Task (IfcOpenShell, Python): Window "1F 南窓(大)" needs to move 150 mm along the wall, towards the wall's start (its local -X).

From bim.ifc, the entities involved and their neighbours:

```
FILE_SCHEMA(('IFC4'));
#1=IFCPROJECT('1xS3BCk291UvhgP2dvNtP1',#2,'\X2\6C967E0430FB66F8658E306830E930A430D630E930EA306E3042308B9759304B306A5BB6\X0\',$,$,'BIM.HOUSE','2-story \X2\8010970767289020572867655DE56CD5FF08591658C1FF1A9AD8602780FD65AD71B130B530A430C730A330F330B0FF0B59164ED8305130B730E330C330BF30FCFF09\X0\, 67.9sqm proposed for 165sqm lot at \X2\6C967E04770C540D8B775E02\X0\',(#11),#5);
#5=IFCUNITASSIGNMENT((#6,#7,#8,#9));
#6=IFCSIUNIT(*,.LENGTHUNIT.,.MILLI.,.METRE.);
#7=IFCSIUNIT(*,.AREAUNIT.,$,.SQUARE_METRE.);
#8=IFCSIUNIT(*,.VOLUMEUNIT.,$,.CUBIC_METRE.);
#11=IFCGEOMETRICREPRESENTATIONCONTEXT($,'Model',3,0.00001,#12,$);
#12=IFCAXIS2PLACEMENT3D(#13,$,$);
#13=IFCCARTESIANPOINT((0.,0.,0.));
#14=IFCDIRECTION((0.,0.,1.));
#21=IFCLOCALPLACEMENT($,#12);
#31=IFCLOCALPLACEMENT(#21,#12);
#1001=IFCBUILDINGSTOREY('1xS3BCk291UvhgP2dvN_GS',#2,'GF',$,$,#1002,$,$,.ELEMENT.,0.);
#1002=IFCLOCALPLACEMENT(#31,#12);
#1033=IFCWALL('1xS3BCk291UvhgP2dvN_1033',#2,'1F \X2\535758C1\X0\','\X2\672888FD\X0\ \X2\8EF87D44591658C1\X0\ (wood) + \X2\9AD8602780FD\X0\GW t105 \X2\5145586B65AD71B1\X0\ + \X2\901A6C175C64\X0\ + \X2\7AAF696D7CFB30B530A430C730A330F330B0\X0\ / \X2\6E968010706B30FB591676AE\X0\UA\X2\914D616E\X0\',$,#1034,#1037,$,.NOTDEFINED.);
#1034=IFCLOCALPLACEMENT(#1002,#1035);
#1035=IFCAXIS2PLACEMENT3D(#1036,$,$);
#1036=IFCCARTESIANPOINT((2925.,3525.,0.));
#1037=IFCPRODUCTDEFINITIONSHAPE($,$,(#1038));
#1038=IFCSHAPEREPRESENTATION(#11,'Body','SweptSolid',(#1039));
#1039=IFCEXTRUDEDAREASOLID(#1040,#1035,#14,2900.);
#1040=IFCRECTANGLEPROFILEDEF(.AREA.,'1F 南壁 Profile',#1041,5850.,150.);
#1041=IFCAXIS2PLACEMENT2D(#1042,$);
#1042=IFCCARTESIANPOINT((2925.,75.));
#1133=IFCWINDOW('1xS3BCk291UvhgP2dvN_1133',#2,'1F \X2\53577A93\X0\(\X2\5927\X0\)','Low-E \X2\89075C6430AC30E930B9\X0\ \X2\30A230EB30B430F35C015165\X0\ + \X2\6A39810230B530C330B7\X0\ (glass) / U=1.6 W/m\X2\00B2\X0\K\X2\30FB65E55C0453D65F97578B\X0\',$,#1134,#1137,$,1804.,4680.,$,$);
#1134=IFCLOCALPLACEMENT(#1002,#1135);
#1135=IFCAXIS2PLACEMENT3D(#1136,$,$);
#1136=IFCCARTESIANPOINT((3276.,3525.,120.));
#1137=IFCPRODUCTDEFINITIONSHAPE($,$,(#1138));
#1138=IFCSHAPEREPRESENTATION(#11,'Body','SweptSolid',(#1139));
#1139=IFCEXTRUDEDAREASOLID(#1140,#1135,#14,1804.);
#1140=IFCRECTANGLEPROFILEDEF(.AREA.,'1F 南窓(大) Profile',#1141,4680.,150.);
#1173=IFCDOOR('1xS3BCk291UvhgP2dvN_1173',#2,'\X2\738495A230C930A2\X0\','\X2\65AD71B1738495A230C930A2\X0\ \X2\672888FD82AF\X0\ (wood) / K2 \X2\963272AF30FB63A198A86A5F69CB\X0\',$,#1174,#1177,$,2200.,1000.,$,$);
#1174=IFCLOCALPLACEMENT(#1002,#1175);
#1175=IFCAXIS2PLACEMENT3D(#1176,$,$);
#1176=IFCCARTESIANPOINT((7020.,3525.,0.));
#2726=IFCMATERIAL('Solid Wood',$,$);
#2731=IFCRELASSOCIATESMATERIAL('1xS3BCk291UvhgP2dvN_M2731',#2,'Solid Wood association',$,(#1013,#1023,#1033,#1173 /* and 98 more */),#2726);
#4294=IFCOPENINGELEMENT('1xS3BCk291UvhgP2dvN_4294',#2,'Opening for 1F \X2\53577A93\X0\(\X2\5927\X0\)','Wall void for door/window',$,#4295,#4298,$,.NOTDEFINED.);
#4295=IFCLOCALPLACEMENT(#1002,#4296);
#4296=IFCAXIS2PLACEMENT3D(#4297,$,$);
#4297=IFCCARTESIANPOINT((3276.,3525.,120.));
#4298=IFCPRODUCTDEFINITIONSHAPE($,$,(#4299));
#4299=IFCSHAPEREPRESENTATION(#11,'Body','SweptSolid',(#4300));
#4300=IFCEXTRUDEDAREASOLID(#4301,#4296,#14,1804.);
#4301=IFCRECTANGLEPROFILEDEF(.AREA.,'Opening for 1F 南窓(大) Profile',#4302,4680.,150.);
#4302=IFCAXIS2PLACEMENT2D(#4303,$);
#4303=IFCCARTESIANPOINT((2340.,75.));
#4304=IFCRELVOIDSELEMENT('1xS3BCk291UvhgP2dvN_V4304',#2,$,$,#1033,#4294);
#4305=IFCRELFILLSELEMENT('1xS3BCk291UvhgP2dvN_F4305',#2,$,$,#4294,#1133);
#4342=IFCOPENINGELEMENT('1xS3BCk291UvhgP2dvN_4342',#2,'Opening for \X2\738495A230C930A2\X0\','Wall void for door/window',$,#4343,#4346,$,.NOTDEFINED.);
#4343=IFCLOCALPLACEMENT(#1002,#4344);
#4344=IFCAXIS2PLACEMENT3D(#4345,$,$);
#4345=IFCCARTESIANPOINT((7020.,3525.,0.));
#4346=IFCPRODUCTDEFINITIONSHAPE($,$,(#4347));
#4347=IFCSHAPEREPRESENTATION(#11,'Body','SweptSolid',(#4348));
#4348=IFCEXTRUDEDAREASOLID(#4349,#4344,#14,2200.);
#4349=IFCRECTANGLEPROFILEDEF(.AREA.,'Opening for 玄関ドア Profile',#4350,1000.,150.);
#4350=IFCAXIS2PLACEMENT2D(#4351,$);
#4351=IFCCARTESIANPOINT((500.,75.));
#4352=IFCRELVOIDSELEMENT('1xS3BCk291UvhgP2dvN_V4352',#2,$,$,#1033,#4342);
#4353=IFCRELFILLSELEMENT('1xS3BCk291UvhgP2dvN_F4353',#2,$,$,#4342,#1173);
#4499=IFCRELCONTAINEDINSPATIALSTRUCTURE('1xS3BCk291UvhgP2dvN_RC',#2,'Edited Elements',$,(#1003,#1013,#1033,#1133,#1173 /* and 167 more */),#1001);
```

```python
import ifcopenshell
import ifcopenshell.api.geometry
import ifcopenshell.util.placement
import ifcopenshell.util.unit

model = ifcopenshell.open("bim.ifc")
unit_scale = ifcopenshell.util.unit.calculate_unit_scale(model)

window = model.by_guid("1xS3BCk291UvhgP2dvN_1133")
opening = window.FillsVoids[0].RelatingOpeningElement
wall = opening.VoidsElements[0].RelatingBuildingElement

wall_matrix = ifcopenshell.util.placement.get_local_placement(wall.ObjectPlacement)
shift = wall_matrix[:3, 0] * -0.15 / unit_scale
before = ifcopenshell.util.placement.get_local_placement(window.ObjectPlacement)[:3, 3].copy()

# The window is not placed relative to its opening, so move both.
for product in (opening, window):
    matrix = ifcopenshell.util.placement.get_local_placement(product.ObjectPlacement)
    matrix[:3, 3] += shift
    ifcopenshell.api.geometry.edit_object_placement(model, product=product, matrix=matrix, is_si=False)

after = ifcopenshell.util.placement.get_local_placement(window.ObjectPlacement)[:3, 3]
print("window moved by", (after - before).round(3) + 0.0)

model.write("bim-out.ifc")
```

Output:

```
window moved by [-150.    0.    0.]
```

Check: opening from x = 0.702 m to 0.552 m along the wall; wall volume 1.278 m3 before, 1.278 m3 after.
